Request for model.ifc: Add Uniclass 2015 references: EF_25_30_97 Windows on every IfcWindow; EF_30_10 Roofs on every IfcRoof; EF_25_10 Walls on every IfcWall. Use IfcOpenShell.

First a look at what the model holds.

```python
import ifcopenshell

model = ifcopenshell.open("model.ifc")
print(model.schema)
print("classifications:", [c.Name for c in model.by_type("IfcClassification")])
for ifc_class in ("IfcDoor", "IfcRoof", "IfcStair", "IfcWall", "IfcWindow"):
    print(ifc_class, len(model.by_type(ifc_class)))
```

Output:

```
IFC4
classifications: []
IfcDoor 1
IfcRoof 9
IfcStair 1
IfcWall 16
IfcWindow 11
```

```python
import ifcopenshell
import ifcopenshell.api.classification

model = ifcopenshell.open("model.ifc")

system = ifcopenshell.api.classification.add_classification(model, classification="Uniclass 2015")

codes = {
    "IfcWindow": ("EF_25_30_97", "Windows"),
    "IfcRoof": ("EF_30_10", "Roofs"),
    "IfcWall": ("EF_25_10", "Walls"),
}
for ifc_class, (code, name) in codes.items():
    products = model.by_type(ifc_class)
    ifcopenshell.api.classification.add_reference(
        model, products=products, classification=system, identification=code, name=name
    )
    print(code, len(products))

model.write("model_edited.ifc")
```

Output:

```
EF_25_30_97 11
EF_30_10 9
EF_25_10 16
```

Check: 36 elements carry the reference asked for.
